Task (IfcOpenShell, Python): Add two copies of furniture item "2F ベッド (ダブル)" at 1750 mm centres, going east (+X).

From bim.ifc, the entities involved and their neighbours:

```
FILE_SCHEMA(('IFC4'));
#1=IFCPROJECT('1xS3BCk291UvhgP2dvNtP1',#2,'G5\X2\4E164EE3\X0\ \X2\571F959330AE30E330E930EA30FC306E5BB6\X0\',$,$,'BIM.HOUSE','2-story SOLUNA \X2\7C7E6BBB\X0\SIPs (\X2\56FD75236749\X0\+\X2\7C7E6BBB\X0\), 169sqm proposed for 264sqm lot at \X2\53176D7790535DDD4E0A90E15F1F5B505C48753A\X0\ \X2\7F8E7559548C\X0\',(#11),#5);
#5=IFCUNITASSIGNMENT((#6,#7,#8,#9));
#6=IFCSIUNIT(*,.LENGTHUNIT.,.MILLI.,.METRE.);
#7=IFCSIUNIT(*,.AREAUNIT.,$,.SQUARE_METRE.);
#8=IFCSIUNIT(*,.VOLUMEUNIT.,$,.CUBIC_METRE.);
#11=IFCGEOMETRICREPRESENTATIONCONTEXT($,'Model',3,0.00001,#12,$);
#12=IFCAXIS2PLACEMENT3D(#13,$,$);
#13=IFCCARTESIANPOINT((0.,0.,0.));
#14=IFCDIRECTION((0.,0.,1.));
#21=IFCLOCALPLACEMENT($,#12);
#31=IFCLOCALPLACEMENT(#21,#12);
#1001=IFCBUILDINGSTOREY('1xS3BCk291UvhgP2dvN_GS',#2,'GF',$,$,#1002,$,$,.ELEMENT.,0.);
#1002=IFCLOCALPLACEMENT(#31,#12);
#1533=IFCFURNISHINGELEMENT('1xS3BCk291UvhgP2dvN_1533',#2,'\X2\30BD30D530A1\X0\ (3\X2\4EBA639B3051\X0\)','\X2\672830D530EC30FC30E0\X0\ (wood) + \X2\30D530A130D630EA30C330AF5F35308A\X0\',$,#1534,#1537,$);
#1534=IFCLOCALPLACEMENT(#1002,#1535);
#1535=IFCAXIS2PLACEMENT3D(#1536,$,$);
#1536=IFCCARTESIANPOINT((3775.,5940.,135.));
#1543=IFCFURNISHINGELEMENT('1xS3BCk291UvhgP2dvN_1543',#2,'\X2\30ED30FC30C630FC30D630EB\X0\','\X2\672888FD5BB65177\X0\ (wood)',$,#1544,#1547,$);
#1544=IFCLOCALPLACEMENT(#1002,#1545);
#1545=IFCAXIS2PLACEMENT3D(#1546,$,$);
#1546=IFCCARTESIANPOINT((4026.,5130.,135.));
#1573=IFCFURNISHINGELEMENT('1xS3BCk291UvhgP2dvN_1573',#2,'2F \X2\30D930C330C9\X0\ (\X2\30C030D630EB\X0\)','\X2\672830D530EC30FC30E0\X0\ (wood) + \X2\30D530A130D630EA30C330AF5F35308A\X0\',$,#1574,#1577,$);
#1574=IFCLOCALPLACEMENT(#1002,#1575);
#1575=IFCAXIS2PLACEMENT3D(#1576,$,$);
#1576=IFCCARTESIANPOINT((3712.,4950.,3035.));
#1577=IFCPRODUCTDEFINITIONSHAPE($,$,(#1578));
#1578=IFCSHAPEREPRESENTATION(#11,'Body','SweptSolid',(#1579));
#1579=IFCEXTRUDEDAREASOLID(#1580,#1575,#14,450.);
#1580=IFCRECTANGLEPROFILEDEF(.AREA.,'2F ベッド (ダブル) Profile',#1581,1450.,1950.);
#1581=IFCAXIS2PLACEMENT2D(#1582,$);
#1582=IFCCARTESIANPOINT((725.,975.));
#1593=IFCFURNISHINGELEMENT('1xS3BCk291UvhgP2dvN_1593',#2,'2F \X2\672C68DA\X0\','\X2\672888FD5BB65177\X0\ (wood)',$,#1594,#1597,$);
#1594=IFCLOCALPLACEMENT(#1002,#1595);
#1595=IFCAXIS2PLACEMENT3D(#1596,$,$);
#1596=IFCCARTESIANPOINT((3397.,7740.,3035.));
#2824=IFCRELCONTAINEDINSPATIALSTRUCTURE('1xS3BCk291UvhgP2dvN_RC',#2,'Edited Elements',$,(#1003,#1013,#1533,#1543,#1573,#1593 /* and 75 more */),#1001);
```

```python
import numpy as np
import ifcopenshell
import ifcopenshell.api.geometry
import ifcopenshell.api.root
import ifcopenshell.util.element
import ifcopenshell.util.placement
import ifcopenshell.util.unit

model = ifcopenshell.open("bim.ifc")
unit_scale = ifcopenshell.util.unit.calculate_unit_scale(model)


def reuse_history(source, copy):
    """copy_class also copies each property set's owner history, people and application; keep the originals."""
    for rel in copy.IsDefinedBy:
        if rel.is_a("IfcRelDefinesByProperties") and (history := rel.RelatingPropertyDefinition.OwnerHistory):
            rel.RelatingPropertyDefinition.OwnerHistory = source.OwnerHistory
            ifcopenshell.util.element.remove_deep2(model, history)


source = model.by_guid("1xS3BCk291UvhgP2dvN_1573")
base = ifcopenshell.util.placement.get_local_placement(source.ObjectPlacement)
step = np.array([1.0, 0.0, 0.0]) * 1.75 / unit_scale

for i in range(1, 3):
    copy = ifcopenshell.api.root.copy_class(model, product=source)
    copy.Representation = ifcopenshell.util.element.copy_deep(
        model, source.Representation, exclude=["IfcGeometricRepresentationContext", "IfcRepresentationMap"]
    )
    reuse_history(source, copy)
    matrix = base.copy()
    matrix[:3, 3] += i * step
    print("added at", matrix[:3, 3].round(3) + 0.0)
    ifcopenshell.api.geometry.edit_object_placement(model, product=copy, matrix=matrix, is_si=False)

model.write("bim_updated.ifc")
```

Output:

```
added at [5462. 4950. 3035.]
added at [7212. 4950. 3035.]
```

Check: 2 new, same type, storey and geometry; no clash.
